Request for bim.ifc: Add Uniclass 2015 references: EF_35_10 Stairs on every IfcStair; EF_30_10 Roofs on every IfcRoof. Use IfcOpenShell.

First a look at what the model holds.

```python
import ifcopenshell

model = ifcopenshell.open("bim.ifc")
print(model.schema)
print("classifications:", [c.Name for c in model.by_type("IfcClassification")])
for ifc_class in ("IfcDoor", "IfcRoof", "IfcStair", "IfcWall", "IfcWindow"):
    print(ifc_class, len(model.by_type(ifc_class)))
```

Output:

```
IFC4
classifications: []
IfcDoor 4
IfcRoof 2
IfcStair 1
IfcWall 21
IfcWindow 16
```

```python
import ifcopenshell
import ifcopenshell.api.classification

model = ifcopenshell.open("bim.ifc")

system = ifcopenshell.api.classification.add_classification(model, classification="Uniclass 2015")

codes = {
    "IfcStair": ("EF_35_10", "Stairs"),
    "IfcRoof": ("EF_30_10", "Roofs"),
}
for ifc_class, (code, name) in codes.items():
    products = model.by_type(ifc_class)
    ifcopenshell.api.classification.add_reference(
        model, products=products, classification=system, identification=code, name=name
    )
    print(code, len(products))

model.write("bim_v2.ifc")
```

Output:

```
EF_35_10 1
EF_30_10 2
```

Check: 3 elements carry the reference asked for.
